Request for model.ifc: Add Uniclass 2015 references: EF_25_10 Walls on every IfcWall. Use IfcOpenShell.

First a look at what the model holds.

```python
import ifcopenshell

model = ifcopenshell.open("model.ifc")
print(model.schema)
print("classifications:", [c.Name for c in model.by_type("IfcClassification")])
for ifc_class in ("IfcDoor", "IfcRoof", "IfcStair", "IfcWall", "IfcWindow"):
    print(ifc_class, len(model.by_type(ifc_class)))
```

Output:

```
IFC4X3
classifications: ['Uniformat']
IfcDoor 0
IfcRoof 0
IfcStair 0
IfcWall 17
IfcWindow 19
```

```python
import ifcopenshell
import ifcopenshell.api.classification

model = ifcopenshell.open("model.ifc")

system = ifcopenshell.api.classification.add_classification(model, classification="Uniclass 2015")

codes = {
    "IfcWall": ("EF_25_10", "Walls"),
}
for ifc_class, (code, name) in codes.items():
    products = model.by_type(ifc_class)
    ifcopenshell.api.classification.add_reference(
        model, products=products, classification=system, identification=code, name=name
    )
    print(code, len(products))

model.write("model_rev.ifc")
```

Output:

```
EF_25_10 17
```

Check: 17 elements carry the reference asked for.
